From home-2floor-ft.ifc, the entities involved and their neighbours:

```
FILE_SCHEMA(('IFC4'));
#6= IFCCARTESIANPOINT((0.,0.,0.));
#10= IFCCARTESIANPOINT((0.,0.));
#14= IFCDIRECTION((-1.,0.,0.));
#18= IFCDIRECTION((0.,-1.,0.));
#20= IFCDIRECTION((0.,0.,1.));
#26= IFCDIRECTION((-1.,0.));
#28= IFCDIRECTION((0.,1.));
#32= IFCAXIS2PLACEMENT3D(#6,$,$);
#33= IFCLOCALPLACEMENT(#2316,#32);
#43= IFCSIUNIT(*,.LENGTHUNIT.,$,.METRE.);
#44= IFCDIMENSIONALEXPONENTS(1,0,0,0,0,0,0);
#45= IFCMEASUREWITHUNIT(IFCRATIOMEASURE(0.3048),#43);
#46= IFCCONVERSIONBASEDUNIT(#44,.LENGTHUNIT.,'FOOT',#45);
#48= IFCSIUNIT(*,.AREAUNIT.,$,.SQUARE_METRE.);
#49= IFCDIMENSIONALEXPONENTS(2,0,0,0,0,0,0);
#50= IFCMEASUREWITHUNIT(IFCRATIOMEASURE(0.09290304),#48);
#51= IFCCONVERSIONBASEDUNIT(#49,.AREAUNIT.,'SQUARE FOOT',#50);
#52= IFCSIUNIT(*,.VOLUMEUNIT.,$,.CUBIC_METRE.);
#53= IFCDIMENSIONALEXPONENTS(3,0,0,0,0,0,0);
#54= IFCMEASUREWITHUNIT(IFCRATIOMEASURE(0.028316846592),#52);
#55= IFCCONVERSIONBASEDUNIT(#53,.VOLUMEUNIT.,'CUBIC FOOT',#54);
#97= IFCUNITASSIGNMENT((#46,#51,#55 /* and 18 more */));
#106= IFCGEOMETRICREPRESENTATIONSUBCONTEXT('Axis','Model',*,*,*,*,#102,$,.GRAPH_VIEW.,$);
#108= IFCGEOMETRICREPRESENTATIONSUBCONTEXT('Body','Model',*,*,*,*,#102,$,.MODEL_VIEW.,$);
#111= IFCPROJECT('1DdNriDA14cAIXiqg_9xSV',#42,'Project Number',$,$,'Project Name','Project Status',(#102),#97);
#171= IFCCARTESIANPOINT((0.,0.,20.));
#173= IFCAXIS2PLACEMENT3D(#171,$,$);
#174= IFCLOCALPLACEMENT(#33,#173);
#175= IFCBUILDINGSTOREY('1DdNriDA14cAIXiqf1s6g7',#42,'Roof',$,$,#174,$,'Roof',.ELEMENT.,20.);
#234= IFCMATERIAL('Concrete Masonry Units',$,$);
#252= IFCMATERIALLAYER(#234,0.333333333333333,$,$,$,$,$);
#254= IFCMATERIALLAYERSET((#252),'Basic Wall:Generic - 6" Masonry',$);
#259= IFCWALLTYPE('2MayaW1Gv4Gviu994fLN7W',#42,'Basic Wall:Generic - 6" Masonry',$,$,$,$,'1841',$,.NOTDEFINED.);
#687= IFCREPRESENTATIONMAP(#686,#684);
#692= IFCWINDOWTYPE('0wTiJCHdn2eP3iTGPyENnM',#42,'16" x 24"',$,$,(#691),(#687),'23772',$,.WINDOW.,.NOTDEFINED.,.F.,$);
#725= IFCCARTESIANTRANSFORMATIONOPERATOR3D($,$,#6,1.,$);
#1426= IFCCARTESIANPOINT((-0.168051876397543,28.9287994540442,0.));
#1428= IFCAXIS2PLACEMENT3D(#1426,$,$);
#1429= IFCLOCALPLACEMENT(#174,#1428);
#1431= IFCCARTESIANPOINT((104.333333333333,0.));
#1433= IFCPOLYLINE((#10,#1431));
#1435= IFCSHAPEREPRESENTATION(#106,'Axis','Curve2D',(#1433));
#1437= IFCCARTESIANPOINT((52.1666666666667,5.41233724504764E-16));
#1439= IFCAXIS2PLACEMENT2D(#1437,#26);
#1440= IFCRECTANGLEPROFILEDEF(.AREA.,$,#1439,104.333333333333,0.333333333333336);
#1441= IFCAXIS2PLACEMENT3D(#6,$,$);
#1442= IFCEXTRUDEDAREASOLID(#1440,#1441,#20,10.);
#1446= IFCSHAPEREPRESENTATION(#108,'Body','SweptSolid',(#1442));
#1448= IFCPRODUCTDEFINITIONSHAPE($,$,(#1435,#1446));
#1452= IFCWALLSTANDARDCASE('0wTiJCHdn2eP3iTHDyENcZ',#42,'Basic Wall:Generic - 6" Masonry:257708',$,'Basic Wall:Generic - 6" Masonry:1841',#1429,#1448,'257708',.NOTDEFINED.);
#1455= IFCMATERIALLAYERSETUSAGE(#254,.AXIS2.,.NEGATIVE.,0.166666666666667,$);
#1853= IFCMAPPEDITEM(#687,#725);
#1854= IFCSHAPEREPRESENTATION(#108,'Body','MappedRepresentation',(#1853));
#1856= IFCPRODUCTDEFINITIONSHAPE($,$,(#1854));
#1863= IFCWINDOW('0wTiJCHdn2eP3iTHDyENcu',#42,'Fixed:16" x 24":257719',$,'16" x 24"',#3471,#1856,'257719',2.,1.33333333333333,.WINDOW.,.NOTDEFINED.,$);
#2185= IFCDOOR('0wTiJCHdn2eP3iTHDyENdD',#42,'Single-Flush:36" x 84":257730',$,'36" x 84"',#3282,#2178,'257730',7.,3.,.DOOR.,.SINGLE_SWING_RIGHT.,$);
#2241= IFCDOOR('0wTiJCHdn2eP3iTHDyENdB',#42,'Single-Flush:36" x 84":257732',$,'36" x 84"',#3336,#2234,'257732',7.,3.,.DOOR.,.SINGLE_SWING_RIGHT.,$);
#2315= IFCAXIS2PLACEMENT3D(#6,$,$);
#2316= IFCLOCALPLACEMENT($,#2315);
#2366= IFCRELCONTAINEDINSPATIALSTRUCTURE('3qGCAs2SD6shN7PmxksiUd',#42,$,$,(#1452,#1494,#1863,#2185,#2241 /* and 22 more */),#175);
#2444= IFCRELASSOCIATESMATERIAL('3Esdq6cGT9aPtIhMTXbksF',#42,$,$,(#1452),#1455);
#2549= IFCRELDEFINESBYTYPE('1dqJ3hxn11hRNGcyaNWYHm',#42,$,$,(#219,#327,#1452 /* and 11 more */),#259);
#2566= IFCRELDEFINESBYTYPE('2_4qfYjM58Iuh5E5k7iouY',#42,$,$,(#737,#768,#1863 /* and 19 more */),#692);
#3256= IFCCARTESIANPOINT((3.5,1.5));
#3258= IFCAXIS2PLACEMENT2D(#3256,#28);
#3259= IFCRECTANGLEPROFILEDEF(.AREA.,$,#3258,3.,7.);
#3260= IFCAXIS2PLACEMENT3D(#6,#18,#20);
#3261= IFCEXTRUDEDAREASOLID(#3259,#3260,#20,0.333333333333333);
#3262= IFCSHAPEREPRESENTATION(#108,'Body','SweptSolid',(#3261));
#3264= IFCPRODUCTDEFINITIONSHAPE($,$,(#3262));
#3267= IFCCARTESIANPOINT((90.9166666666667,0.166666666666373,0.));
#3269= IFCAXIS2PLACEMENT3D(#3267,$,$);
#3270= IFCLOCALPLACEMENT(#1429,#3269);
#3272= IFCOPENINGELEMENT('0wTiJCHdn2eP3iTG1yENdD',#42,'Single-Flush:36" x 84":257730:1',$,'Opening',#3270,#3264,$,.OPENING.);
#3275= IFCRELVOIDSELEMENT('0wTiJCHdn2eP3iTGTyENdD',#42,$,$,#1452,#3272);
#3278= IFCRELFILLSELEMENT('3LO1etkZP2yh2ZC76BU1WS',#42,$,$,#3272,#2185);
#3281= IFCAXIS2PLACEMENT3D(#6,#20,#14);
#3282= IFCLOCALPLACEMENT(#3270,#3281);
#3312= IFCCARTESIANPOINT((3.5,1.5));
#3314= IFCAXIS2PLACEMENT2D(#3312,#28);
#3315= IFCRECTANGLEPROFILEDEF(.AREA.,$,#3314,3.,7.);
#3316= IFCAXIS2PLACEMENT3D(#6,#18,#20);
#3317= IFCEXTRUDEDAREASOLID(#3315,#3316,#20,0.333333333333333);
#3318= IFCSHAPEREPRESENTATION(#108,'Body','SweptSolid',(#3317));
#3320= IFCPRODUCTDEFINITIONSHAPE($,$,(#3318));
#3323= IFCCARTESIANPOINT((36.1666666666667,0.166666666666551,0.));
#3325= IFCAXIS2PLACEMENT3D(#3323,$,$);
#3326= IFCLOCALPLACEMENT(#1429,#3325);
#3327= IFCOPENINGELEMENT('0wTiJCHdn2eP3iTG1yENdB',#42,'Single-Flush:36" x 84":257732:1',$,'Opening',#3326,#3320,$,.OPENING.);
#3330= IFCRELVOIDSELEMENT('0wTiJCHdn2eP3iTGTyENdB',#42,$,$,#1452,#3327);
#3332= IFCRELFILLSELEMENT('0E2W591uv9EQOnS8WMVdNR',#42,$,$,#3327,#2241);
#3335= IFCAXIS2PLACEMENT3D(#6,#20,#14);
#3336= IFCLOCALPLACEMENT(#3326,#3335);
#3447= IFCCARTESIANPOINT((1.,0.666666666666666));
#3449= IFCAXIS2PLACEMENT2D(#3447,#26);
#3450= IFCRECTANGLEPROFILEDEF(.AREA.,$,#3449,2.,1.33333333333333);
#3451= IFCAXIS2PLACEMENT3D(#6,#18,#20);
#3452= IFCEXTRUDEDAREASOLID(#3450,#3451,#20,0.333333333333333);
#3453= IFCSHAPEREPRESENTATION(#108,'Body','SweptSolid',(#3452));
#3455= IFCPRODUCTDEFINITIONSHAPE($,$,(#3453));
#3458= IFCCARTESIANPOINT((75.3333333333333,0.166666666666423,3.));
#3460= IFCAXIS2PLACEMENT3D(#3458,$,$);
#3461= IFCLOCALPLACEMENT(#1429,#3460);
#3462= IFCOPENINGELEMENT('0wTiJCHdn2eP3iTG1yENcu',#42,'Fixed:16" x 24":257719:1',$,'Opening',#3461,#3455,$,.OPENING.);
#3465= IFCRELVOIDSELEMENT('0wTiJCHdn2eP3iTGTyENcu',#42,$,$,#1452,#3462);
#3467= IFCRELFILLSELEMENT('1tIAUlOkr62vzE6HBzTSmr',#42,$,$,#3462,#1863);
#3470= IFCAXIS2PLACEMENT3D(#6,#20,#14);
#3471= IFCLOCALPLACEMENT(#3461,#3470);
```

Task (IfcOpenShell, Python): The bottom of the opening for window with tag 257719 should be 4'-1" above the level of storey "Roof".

```python
import numpy as np
import ifcopenshell
import ifcopenshell.api.geometry
import ifcopenshell.geom
import ifcopenshell.util.element
import ifcopenshell.util.placement
import ifcopenshell.util.shape
import ifcopenshell.util.unit

model = ifcopenshell.open("home-2floor-ft.ifc")
unit_scale = ifcopenshell.util.unit.calculate_unit_scale(model)

window = model.by_id(1863)
opening = window.FillsVoids[0].RelatingOpeningElement
storey = ifcopenshell.util.element.get_container(window, ifc_class="IfcBuildingStorey")
level = ifcopenshell.util.placement.get_local_placement(storey.ObjectPlacement)[2, 3]

# The opening's origin need not be at the sill, so measure its lowest point.
shape = ifcopenshell.geom.create_shape(ifcopenshell.geom.settings(), opening)
bottom = ifcopenshell.util.shape.get_shape_bottom_elevation(shape, shape.geometry) / unit_scale
dz = level + 49 * 0.0254 / unit_scale - bottom

shift = np.array([0.0, 0.0, dz])
# The window is placed relative to its opening, so it follows when the opening moves.
matrix = ifcopenshell.util.placement.get_local_placement(opening.ObjectPlacement)
matrix[:3, 3] += shift
ifcopenshell.api.geometry.edit_object_placement(
    model, product=opening, matrix=matrix, is_si=False, should_transform_children=True
)

print(f"moved by {dz * unit_scale:+.3f} m")

model.write("home-2floor-ft_updated.ifc")
```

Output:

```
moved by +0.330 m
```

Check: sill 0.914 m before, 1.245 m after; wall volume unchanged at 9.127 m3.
